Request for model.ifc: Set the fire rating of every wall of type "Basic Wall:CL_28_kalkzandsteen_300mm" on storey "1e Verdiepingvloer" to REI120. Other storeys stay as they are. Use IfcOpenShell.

First a look at what the model holds.

```python
import ifcopenshell
import ifcopenshell.util.element

model = ifcopenshell.open("model.ifc")
print(model.schema)
storey = next(s for s in model.by_type("IfcBuildingStorey") if s.Name == "1e Verdiepingvloer")
walls = [e for e in ifcopenshell.util.element.get_decomposition(storey) if e.is_a("IfcWall")]
seen = {}
for e in walls:
    element_type = ifcopenshell.util.element.get_type(e)
    key = (element_type.Name if element_type != e and element_type else None, ifcopenshell.util.element.get_pset(e, "Pset_WallCommon", "FireRating"))
    seen[key] = seen.get(key, 0) + 1
for (name, value), count in sorted(seen.items(), key=str):
    print(count, "x", name, "|", value)
```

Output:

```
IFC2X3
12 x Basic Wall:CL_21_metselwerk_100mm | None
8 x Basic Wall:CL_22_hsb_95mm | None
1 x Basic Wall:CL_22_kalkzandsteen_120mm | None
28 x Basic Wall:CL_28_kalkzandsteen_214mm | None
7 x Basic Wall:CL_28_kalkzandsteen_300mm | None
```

```python
import ifcopenshell
import ifcopenshell.api.pset
import ifcopenshell.util.element

model = ifcopenshell.open("model.ifc")

storey = next(s for s in model.by_type("IfcBuildingStorey") if s.Name == "1e Verdiepingvloer")
walls = [e for e in ifcopenshell.util.element.get_decomposition(storey) if e.is_a("IfcWall")]

count = 0
for e in walls:
    element_type = ifcopenshell.util.element.get_type(e)
    if element_type in (None, e) or element_type.Name != "Basic Wall:CL_28_kalkzandsteen_300mm":
        continue
    # add_pset returns the element's existing set when there is one.
    pset = ifcopenshell.api.pset.add_pset(model, product=e, name="Pset_WallCommon")
    ifcopenshell.api.pset.edit_pset(model, pset=pset, properties={"FireRating": "REI120"})
    count += 1

print(count, "walls updated")

model.write("model_edited.ifc")
```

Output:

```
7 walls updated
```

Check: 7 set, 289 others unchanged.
